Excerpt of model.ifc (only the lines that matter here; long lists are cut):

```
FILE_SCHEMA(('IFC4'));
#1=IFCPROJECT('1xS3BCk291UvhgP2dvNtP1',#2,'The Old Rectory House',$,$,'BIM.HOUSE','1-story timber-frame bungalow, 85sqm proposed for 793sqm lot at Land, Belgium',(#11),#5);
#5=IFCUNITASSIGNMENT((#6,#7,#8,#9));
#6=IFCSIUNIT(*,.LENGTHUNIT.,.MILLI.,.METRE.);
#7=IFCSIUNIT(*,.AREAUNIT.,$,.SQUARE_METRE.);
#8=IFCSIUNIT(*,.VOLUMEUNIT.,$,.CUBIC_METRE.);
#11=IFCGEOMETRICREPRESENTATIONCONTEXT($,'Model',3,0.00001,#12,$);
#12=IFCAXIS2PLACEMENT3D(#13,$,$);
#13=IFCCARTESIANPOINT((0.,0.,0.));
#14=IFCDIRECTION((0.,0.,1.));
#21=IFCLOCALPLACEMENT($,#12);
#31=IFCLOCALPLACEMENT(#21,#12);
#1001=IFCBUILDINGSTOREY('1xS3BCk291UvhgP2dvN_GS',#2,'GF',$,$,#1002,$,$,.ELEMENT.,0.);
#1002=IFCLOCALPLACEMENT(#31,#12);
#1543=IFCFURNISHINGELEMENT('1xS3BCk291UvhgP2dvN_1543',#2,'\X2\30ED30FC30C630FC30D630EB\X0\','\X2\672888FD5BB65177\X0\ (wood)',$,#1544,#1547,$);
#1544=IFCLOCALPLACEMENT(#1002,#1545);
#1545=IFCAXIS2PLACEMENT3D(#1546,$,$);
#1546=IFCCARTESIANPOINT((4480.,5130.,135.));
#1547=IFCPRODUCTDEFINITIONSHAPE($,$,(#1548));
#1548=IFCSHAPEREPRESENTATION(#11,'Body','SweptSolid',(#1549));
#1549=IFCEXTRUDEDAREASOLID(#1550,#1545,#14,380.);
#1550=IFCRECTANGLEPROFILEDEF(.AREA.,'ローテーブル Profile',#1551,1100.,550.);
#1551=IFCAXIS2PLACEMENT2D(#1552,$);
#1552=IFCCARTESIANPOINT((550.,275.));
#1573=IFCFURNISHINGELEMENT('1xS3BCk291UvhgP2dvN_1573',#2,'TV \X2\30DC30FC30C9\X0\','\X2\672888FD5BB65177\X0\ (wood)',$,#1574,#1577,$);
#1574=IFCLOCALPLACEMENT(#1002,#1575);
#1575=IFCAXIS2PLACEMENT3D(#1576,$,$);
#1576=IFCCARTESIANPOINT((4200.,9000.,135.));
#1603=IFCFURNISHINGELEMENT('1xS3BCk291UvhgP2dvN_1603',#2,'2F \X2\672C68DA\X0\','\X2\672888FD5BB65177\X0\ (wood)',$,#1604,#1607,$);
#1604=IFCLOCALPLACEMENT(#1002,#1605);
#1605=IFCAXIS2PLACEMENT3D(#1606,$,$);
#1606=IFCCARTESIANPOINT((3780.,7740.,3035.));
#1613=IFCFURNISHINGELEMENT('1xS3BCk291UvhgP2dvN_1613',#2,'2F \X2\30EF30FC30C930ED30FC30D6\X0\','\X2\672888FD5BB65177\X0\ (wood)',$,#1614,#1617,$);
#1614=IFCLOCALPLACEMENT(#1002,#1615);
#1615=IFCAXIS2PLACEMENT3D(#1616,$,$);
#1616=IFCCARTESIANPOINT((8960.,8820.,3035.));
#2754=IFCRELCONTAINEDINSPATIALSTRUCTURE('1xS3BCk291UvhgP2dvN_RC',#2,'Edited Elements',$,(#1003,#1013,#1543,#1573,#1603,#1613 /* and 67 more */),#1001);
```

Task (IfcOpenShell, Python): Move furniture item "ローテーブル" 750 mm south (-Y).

```python
import ifcopenshell
import ifcopenshell.api.geometry
import ifcopenshell.util.placement
import ifcopenshell.util.unit

model = ifcopenshell.open("model.ifc")
unit_scale = ifcopenshell.util.unit.calculate_unit_scale(model)

item = model.by_guid("1xS3BCk291UvhgP2dvN_1543")
matrix = ifcopenshell.util.placement.get_local_placement(item.ObjectPlacement)
matrix[1, 3] -= 0.75 / unit_scale
ifcopenshell.api.geometry.edit_object_placement(model, product=item, matrix=matrix, is_si=False)

print(ifcopenshell.util.placement.get_local_placement(item.ObjectPlacement).round(3) + 0.0)

model.write("model-out.ifc")
```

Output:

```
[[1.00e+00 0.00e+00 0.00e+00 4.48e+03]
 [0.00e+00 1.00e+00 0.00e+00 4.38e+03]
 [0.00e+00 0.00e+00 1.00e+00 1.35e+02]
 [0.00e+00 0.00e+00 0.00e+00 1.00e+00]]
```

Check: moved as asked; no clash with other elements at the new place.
